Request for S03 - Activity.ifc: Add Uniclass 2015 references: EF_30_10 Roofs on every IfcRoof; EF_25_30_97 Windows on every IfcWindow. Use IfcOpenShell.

First a look at what the model holds.

```python
import ifcopenshell

model = ifcopenshell.open("S03 - Activity.ifc")
print(model.schema)
print("classifications:", [c.Name for c in model.by_type("IfcClassification")])
for ifc_class in ("IfcDoor", "IfcRoof", "IfcStair", "IfcWall", "IfcWindow"):
    print(ifc_class, len(model.by_type(ifc_class)))
```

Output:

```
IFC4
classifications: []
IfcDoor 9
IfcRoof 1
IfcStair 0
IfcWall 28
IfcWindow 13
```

```python
import ifcopenshell
import ifcopenshell.api.classification

model = ifcopenshell.open("S03 - Activity.ifc")

system = ifcopenshell.api.classification.add_classification(model, classification="Uniclass 2015")

codes = {
    "IfcRoof": ("EF_30_10", "Roofs"),
    "IfcWindow": ("EF_25_30_97", "Windows"),
}
for ifc_class, (code, name) in codes.items():
    products = model.by_type(ifc_class)
    ifcopenshell.api.classification.add_reference(
        model, products=products, classification=system, identification=code, name=name
    )
    print(code, len(products))

model.write("S03 - Activity_rev.ifc")
```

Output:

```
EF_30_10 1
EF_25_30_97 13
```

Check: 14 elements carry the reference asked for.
